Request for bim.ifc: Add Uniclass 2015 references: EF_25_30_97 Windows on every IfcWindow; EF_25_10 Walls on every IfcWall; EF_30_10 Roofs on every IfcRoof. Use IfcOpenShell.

First a look at what the model holds.

```python
import ifcopenshell

model = ifcopenshell.open("bim.ifc")
print(model.schema)
print("classifications:", [c.Name for c in model.by_type("IfcClassification")])
for ifc_class in ("IfcDoor", "IfcRoof", "IfcStair", "IfcWall", "IfcWindow"):
    print(ifc_class, len(model.by_type(ifc_class)))
```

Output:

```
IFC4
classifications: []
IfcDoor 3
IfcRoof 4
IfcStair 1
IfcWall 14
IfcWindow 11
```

```python
import ifcopenshell
import ifcopenshell.api.classification

model = ifcopenshell.open("bim.ifc")

system = ifcopenshell.api.classification.add_classification(model, classification="Uniclass 2015")

codes = {
    "IfcWindow": ("EF_25_30_97", "Windows"),
    "IfcWall": ("EF_25_10", "Walls"),
    "IfcRoof": ("EF_30_10", "Roofs"),
}
for ifc_class, (code, name) in codes.items():
    products = model.by_type(ifc_class)
    ifcopenshell.api.classification.add_reference(
        model, products=products, classification=system, identification=code, name=name
    )
    print(code, len(products))

model.write("bim_edited.ifc")
```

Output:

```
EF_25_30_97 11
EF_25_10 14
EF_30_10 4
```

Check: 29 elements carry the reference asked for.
